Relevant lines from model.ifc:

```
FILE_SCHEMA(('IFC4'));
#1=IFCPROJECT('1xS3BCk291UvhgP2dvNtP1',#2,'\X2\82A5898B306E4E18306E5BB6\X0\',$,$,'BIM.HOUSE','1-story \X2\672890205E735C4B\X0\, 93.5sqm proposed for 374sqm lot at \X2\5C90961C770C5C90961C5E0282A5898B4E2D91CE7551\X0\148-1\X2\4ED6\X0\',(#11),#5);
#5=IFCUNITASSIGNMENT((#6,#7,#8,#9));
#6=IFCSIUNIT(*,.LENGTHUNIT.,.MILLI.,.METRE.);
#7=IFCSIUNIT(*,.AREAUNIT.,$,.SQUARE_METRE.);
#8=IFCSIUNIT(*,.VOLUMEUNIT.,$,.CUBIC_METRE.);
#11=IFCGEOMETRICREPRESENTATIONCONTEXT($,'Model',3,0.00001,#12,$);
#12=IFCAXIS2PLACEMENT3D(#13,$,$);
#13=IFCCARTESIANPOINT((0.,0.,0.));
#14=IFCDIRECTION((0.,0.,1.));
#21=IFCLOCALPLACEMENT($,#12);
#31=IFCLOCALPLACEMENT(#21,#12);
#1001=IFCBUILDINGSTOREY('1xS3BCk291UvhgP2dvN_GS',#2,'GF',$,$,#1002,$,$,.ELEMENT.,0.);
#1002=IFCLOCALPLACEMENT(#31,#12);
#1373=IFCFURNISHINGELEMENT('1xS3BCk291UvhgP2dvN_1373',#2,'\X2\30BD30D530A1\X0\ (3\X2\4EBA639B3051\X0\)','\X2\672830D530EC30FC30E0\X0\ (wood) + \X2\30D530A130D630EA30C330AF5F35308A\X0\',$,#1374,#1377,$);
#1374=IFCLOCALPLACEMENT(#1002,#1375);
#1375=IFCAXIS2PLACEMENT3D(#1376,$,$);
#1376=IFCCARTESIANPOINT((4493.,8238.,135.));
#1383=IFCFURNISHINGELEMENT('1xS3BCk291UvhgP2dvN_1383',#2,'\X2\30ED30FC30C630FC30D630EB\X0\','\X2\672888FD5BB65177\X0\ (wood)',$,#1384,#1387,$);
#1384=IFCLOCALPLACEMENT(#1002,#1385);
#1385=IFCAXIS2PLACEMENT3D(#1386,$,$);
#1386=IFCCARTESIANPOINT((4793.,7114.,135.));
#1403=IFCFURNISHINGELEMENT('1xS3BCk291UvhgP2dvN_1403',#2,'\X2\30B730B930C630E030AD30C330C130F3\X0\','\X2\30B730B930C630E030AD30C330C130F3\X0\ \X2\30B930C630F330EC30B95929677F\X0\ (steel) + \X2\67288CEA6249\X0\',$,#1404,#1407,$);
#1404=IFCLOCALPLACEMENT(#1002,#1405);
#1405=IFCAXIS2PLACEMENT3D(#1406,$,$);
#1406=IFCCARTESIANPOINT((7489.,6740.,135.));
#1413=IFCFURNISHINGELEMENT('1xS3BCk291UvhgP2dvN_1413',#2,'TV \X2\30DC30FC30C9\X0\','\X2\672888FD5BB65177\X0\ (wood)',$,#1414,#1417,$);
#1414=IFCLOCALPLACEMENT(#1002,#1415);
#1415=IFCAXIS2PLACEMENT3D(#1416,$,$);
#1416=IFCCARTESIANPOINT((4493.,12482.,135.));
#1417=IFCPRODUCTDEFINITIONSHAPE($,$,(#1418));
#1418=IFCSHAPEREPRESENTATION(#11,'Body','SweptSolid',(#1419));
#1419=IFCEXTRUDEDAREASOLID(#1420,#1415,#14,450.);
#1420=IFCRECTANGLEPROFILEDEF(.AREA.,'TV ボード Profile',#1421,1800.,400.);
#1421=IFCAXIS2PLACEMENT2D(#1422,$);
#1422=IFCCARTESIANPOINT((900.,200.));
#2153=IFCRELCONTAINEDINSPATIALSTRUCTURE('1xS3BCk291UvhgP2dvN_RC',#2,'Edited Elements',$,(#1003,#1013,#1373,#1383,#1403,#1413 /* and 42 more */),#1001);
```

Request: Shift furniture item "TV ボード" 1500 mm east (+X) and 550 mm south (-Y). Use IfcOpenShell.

```python
import ifcopenshell
import ifcopenshell.api.geometry
import ifcopenshell.util.placement

model = ifcopenshell.open("model.ifc")

item = model.by_guid("1xS3BCk291UvhgP2dvN_1413")
matrix = ifcopenshell.util.placement.get_local_placement(item.ObjectPlacement)
matrix[0, 3] += 1500.0
matrix[1, 3] -= 550.0
ifcopenshell.api.geometry.edit_object_placement(model, product=item, matrix=matrix, is_si=False)

print(ifcopenshell.util.placement.get_local_placement(item.ObjectPlacement).round(3) + 0.0)

model.write("model_updated.ifc")
```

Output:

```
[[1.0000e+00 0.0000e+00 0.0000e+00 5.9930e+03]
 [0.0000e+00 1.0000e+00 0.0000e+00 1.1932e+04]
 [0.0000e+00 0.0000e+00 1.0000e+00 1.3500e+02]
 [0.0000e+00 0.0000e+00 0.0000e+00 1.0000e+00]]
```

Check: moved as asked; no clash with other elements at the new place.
